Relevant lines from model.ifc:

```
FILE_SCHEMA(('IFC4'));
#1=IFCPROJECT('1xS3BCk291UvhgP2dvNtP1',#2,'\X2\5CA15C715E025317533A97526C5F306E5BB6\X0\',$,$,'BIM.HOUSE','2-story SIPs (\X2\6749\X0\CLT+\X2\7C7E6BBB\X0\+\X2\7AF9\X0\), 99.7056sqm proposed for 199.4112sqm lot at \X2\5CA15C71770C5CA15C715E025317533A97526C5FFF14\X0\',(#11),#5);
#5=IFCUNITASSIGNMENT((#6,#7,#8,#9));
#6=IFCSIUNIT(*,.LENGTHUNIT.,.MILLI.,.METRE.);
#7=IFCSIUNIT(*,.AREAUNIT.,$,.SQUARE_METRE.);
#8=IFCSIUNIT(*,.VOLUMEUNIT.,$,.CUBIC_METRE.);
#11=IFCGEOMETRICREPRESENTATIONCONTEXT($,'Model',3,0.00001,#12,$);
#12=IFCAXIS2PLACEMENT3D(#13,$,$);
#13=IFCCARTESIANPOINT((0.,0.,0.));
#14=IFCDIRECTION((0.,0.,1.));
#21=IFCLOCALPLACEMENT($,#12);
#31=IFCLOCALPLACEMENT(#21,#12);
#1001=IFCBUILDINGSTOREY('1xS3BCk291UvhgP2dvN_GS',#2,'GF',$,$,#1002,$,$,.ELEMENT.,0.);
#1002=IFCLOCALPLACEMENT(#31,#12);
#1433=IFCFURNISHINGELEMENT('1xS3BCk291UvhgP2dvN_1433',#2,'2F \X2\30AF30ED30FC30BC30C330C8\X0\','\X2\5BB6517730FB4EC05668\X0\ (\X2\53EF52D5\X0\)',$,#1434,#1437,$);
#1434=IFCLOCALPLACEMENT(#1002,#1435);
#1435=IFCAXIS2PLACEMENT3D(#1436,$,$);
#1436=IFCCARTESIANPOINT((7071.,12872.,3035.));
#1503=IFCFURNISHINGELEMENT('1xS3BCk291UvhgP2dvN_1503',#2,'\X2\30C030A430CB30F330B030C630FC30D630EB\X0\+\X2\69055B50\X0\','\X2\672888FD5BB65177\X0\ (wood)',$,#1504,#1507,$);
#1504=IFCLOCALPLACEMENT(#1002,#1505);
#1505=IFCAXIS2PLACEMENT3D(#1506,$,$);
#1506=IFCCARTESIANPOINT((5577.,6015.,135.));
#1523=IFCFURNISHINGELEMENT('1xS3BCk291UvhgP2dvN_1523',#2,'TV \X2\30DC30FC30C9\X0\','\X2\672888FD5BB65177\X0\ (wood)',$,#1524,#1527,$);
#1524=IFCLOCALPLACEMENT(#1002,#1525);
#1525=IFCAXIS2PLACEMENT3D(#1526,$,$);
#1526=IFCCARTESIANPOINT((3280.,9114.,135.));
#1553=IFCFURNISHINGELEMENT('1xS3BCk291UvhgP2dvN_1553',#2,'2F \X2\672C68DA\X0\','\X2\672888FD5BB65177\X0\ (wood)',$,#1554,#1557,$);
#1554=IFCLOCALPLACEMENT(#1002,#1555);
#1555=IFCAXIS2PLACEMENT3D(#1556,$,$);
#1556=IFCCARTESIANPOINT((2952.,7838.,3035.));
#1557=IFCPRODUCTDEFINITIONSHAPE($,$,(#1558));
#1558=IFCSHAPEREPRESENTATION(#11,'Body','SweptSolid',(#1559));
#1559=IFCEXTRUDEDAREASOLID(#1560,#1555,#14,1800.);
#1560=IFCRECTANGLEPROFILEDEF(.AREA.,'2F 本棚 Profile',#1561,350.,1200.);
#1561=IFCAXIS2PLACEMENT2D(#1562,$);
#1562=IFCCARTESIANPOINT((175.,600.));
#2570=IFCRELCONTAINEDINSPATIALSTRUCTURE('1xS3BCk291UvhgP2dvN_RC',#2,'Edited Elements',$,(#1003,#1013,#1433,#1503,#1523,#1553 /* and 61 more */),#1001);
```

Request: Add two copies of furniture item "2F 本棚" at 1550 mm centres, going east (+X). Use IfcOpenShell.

```python
import numpy as np
import ifcopenshell
import ifcopenshell.api.geometry
import ifcopenshell.api.root
import ifcopenshell.util.element
import ifcopenshell.util.placement
import ifcopenshell.util.unit

model = ifcopenshell.open("model.ifc")
unit_scale = ifcopenshell.util.unit.calculate_unit_scale(model)


def reuse_history(source, copy):
    """copy_class also copies each property set's owner history, people and application; keep the originals."""
    for rel in copy.IsDefinedBy:
        if rel.is_a("IfcRelDefinesByProperties") and (history := rel.RelatingPropertyDefinition.OwnerHistory):
            rel.RelatingPropertyDefinition.OwnerHistory = source.OwnerHistory
            ifcopenshell.util.element.remove_deep2(model, history)


source = model.by_guid("1xS3BCk291UvhgP2dvN_1553")
base = ifcopenshell.util.placement.get_local_placement(source.ObjectPlacement)
step = np.array([1.0, 0.0, 0.0]) * 1.55 / unit_scale

for i in range(1, 3):
    copy = ifcopenshell.api.root.copy_class(model, product=source)
    copy.Representation = ifcopenshell.util.element.copy_deep(
        model, source.Representation, exclude=["IfcGeometricRepresentationContext", "IfcRepresentationMap"]
    )
    reuse_history(source, copy)
    matrix = base.copy()
    matrix[:3, 3] += i * step
    print("added at", matrix[:3, 3].round(3) + 0.0)
    ifcopenshell.api.geometry.edit_object_placement(model, product=copy, matrix=matrix, is_si=False)

model.write("model_updated.ifc")
```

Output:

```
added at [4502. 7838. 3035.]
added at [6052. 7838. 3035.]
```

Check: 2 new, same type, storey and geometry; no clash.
